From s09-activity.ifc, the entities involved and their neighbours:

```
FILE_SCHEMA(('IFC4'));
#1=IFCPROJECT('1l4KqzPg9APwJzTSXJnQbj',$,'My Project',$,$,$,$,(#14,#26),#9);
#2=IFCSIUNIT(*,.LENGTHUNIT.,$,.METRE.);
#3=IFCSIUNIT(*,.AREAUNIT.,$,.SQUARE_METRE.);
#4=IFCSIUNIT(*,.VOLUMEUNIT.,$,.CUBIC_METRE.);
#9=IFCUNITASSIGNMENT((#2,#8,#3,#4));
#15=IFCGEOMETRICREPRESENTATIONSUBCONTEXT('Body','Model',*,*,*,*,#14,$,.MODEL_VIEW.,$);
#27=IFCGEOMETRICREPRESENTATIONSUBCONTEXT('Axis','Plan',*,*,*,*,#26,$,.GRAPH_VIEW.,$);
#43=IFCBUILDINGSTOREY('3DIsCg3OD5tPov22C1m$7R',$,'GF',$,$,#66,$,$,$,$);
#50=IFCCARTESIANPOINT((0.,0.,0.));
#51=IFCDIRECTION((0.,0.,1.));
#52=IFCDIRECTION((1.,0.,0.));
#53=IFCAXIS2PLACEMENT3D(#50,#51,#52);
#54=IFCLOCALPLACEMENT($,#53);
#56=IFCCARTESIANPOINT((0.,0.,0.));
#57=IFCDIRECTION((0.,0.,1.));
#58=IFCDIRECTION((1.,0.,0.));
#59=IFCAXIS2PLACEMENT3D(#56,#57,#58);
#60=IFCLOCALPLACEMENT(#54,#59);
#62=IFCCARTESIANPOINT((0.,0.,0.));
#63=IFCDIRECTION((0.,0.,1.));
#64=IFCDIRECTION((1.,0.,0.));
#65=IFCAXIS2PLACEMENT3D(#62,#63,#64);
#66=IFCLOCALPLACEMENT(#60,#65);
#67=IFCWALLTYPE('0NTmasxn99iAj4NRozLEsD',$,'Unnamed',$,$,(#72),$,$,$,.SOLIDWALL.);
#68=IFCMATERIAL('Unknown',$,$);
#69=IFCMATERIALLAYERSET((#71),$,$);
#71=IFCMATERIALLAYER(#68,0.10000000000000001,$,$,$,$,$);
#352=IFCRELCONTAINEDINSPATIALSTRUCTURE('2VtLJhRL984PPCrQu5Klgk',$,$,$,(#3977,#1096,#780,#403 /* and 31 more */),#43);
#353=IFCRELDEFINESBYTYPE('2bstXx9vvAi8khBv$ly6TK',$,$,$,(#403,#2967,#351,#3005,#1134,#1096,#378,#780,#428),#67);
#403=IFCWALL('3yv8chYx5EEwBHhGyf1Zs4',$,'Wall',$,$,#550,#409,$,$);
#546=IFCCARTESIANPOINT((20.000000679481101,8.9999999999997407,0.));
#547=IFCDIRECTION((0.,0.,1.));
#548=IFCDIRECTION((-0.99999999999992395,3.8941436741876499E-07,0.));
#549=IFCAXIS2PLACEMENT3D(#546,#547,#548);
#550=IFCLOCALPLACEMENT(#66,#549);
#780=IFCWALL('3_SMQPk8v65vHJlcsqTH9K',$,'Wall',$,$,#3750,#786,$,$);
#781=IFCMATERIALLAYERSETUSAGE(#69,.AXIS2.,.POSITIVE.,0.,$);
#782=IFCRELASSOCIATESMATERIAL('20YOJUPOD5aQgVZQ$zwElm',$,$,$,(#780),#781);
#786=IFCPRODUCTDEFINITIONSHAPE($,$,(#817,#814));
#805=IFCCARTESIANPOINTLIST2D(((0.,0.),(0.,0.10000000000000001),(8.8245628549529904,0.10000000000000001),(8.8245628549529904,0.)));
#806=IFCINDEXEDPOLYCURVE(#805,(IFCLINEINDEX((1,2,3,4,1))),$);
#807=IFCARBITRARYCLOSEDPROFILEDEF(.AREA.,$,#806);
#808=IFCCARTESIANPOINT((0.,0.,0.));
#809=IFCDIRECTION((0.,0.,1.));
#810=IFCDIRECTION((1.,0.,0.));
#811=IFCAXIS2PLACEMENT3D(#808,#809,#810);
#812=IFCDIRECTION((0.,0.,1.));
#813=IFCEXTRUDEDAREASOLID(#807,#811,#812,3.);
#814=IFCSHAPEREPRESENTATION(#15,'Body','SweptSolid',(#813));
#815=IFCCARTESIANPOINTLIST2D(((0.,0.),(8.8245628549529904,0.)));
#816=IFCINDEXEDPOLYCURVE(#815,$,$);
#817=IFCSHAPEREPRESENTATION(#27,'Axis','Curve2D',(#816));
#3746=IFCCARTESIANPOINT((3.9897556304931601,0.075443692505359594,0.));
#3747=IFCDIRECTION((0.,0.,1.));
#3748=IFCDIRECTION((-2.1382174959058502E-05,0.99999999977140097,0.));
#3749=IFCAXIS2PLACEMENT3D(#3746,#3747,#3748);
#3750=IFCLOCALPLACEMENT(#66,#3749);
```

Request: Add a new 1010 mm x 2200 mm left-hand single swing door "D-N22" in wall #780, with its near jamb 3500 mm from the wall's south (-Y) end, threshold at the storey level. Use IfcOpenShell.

```python
import numpy as np
import ifcopenshell
import ifcopenshell.api.feature
import ifcopenshell.api.geometry
import ifcopenshell.api.root
import ifcopenshell.api.spatial
import ifcopenshell.geom
import ifcopenshell.util.element
import ifcopenshell.util.placement
import ifcopenshell.util.representation
import ifcopenshell.util.shape
import ifcopenshell.util.unit

model = ifcopenshell.open("s09-activity.ifc")
unit_scale = ifcopenshell.util.unit.calculate_unit_scale(model)
settings = ifcopenshell.geom.settings()


def volume(element):
    """Net volume in cubic metres, openings subtracted."""
    shape = ifcopenshell.geom.create_shape(settings, element)
    return ifcopenshell.util.shape.get_volume(shape.geometry)


wall = model.by_id(780)
storey = ifcopenshell.util.element.get_container(wall, ifc_class="IfcBuildingStorey")
context = ifcopenshell.util.representation.get_context(model, "Model", "Body", "MODEL_VIEW")
before = volume(wall)

width, height, from_end, sill = 1.01, 2.2, 3.5, 0.0  # metres

# The wall runs along its own X axis, and the end named is its -X end.
wall_shape = ifcopenshell.geom.create_shape(settings, wall)
x, y, z = ifcopenshell.util.shape.get_vertices(wall_shape.geometry).T
start = x.min() + from_end
face, thickness = float(y.min()), float(y.max() - y.min())
wall_matrix = ifcopenshell.util.placement.get_local_placement(wall.ObjectPlacement)
level = ifcopenshell.util.placement.get_local_placement(storey.ObjectPlacement)[2, 3]


def in_wall(x, y):
    """Placement at x, y metres in the wall's axes, at sill height."""
    matrix = wall_matrix.copy()
    matrix[:, 3] = wall_matrix @ np.array([x / unit_scale, y / unit_scale, 0.0, 1.0])
    matrix[2, 3] = level + sill / unit_scale
    return matrix


# Opening: a box that overshoots both wall faces by 50 mm.
opening = ifcopenshell.api.root.create_entity(model, ifc_class="IfcOpeningElement", predefined_type="OPENING")
box = ifcopenshell.api.geometry.add_wall_representation(
    model, context=context, length=width, height=height, thickness=thickness + 0.1
)
ifcopenshell.api.geometry.assign_representation(model, product=opening, representation=box)
ifcopenshell.api.geometry.edit_object_placement(model, product=opening, matrix=in_wall(start, face - 0.05), is_si=False)
ifcopenshell.api.feature.add_feature(model, feature=opening, element=wall)

door = ifcopenshell.api.root.create_entity(model, ifc_class="IfcDoor", name="D-N22", predefined_type="DOOR")
door.OverallWidth, door.OverallHeight = width / unit_scale, height / unit_scale
door.OperationType = "SINGLE_SWING_LEFT"
body = ifcopenshell.api.geometry.add_door_representation(
    model,
    context=context,
    overall_width=door.OverallWidth,
    overall_height=door.OverallHeight,
    operation_type="SINGLE_SWING_LEFT",
    lining_properties={"LiningDepth": thickness / unit_scale, "ThresholdDepth": thickness / unit_scale},
)
ifcopenshell.api.geometry.assign_representation(model, product=door, representation=body)
ifcopenshell.api.spatial.assign_container(model, products=[door], relating_structure=storey)
ifcopenshell.api.feature.add_filling(model, opening=opening, element=door)

# The lining spans the wall, so the door starts at the wall face.
ifcopenshell.api.geometry.edit_object_placement(model, product=door, matrix=in_wall(start, face), is_si=False)

after = volume(wall)

print(f"wall volume {before:.3f} -> {after:.3f} m3")

model.write("s09-activity-out.ifc")
```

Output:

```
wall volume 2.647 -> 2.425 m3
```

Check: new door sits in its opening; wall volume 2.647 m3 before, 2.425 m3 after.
